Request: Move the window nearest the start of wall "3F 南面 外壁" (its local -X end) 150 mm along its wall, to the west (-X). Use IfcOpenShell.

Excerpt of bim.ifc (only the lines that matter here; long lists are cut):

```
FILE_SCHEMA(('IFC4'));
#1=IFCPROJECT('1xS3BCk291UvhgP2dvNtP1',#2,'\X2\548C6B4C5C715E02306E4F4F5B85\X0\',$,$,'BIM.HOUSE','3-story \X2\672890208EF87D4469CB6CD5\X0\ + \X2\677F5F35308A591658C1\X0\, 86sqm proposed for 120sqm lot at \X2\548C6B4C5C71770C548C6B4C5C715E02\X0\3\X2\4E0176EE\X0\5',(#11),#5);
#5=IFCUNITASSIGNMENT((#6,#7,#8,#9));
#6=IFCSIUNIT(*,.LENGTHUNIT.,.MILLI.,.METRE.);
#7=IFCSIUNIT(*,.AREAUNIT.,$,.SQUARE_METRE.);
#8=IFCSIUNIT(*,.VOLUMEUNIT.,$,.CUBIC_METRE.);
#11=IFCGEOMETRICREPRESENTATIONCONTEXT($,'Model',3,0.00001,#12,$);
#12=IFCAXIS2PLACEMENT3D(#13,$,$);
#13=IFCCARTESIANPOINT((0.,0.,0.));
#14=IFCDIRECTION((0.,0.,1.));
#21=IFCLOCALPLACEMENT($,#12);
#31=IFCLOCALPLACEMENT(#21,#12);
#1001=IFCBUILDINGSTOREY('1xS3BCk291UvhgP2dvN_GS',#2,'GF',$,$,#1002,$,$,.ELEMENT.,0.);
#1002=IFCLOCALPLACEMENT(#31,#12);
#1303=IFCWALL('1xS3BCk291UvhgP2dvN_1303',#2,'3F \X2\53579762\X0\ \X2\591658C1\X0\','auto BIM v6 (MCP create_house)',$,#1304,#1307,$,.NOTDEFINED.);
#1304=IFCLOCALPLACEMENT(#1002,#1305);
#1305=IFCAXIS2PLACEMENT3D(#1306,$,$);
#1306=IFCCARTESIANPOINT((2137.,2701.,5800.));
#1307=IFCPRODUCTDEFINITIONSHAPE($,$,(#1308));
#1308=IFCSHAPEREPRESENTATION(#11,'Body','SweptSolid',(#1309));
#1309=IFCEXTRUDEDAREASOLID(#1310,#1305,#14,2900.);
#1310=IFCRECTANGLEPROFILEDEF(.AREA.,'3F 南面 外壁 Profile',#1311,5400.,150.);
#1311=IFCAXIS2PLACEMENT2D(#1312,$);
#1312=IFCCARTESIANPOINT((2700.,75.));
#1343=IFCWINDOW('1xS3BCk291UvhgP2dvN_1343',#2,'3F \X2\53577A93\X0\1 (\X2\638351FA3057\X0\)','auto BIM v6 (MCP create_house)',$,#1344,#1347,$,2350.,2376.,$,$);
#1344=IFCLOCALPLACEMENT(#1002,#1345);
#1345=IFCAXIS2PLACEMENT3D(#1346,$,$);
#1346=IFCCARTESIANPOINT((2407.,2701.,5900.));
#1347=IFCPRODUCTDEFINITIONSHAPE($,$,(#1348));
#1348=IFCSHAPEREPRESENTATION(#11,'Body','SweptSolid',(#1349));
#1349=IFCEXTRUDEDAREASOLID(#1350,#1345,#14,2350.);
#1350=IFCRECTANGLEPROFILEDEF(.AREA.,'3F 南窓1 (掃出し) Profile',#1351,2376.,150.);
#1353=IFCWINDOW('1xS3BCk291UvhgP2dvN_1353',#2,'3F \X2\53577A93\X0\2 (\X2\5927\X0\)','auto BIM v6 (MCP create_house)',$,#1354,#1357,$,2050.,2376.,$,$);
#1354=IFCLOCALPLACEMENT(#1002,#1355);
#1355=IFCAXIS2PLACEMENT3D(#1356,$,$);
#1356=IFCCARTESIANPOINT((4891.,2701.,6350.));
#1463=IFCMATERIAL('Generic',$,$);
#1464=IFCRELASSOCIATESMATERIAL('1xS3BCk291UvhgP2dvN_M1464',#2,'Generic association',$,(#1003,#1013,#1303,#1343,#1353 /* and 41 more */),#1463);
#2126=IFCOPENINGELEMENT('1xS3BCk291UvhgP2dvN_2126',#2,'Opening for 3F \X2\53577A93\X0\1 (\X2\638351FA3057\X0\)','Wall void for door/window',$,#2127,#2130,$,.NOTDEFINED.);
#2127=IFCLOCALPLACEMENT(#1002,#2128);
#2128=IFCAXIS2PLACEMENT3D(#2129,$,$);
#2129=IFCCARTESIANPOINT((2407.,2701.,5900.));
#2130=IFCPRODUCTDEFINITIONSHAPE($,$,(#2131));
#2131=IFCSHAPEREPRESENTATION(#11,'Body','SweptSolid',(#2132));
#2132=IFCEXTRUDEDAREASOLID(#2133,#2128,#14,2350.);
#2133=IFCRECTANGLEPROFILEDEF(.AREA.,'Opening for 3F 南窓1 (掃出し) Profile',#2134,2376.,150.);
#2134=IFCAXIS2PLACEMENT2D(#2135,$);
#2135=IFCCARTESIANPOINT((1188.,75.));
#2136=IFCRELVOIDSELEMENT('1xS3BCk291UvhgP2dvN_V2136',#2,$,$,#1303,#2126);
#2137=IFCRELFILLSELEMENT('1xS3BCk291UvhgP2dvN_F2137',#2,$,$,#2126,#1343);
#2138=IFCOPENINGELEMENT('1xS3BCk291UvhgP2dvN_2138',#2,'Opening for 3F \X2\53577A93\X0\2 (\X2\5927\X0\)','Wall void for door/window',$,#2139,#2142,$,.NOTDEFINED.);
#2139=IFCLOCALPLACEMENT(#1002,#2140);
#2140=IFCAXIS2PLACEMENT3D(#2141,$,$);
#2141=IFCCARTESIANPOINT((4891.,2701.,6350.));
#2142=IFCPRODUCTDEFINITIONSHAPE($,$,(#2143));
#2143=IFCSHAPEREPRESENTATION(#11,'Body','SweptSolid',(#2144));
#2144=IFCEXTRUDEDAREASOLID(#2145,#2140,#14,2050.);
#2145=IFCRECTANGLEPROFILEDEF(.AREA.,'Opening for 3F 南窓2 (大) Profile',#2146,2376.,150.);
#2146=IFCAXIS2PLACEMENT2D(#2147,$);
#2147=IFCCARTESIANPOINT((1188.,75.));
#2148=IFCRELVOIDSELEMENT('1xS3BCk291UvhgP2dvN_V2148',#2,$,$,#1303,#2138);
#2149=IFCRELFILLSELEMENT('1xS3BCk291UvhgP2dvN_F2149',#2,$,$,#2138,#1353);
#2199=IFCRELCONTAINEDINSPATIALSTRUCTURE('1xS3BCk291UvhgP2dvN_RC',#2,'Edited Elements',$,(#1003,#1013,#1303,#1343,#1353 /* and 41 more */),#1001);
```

```python
import ifcopenshell
import ifcopenshell.api.geometry
import ifcopenshell.util.placement

model = ifcopenshell.open("bim.ifc")

window = model.by_id(1343)
opening = window.FillsVoids[0].RelatingOpeningElement
wall = opening.VoidsElements[0].RelatingBuildingElement

wall_matrix = ifcopenshell.util.placement.get_local_placement(wall.ObjectPlacement)
shift = wall_matrix[:3, 0] * -150.0
before = ifcopenshell.util.placement.get_local_placement(window.ObjectPlacement)[:3, 3].copy()

# The window is not placed relative to its opening, so move both.
for product in (opening, window):
    matrix = ifcopenshell.util.placement.get_local_placement(product.ObjectPlacement)
    matrix[:3, 3] += shift
    ifcopenshell.api.geometry.edit_object_placement(model, product=product, matrix=matrix, is_si=False)

after = ifcopenshell.util.placement.get_local_placement(window.ObjectPlacement)[:3, 3]
print("window moved by", (after - before).round(3) + 0.0)

model.write("bim_rev.ifc")
```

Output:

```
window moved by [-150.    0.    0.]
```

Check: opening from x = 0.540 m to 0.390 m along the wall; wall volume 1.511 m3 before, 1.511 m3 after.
